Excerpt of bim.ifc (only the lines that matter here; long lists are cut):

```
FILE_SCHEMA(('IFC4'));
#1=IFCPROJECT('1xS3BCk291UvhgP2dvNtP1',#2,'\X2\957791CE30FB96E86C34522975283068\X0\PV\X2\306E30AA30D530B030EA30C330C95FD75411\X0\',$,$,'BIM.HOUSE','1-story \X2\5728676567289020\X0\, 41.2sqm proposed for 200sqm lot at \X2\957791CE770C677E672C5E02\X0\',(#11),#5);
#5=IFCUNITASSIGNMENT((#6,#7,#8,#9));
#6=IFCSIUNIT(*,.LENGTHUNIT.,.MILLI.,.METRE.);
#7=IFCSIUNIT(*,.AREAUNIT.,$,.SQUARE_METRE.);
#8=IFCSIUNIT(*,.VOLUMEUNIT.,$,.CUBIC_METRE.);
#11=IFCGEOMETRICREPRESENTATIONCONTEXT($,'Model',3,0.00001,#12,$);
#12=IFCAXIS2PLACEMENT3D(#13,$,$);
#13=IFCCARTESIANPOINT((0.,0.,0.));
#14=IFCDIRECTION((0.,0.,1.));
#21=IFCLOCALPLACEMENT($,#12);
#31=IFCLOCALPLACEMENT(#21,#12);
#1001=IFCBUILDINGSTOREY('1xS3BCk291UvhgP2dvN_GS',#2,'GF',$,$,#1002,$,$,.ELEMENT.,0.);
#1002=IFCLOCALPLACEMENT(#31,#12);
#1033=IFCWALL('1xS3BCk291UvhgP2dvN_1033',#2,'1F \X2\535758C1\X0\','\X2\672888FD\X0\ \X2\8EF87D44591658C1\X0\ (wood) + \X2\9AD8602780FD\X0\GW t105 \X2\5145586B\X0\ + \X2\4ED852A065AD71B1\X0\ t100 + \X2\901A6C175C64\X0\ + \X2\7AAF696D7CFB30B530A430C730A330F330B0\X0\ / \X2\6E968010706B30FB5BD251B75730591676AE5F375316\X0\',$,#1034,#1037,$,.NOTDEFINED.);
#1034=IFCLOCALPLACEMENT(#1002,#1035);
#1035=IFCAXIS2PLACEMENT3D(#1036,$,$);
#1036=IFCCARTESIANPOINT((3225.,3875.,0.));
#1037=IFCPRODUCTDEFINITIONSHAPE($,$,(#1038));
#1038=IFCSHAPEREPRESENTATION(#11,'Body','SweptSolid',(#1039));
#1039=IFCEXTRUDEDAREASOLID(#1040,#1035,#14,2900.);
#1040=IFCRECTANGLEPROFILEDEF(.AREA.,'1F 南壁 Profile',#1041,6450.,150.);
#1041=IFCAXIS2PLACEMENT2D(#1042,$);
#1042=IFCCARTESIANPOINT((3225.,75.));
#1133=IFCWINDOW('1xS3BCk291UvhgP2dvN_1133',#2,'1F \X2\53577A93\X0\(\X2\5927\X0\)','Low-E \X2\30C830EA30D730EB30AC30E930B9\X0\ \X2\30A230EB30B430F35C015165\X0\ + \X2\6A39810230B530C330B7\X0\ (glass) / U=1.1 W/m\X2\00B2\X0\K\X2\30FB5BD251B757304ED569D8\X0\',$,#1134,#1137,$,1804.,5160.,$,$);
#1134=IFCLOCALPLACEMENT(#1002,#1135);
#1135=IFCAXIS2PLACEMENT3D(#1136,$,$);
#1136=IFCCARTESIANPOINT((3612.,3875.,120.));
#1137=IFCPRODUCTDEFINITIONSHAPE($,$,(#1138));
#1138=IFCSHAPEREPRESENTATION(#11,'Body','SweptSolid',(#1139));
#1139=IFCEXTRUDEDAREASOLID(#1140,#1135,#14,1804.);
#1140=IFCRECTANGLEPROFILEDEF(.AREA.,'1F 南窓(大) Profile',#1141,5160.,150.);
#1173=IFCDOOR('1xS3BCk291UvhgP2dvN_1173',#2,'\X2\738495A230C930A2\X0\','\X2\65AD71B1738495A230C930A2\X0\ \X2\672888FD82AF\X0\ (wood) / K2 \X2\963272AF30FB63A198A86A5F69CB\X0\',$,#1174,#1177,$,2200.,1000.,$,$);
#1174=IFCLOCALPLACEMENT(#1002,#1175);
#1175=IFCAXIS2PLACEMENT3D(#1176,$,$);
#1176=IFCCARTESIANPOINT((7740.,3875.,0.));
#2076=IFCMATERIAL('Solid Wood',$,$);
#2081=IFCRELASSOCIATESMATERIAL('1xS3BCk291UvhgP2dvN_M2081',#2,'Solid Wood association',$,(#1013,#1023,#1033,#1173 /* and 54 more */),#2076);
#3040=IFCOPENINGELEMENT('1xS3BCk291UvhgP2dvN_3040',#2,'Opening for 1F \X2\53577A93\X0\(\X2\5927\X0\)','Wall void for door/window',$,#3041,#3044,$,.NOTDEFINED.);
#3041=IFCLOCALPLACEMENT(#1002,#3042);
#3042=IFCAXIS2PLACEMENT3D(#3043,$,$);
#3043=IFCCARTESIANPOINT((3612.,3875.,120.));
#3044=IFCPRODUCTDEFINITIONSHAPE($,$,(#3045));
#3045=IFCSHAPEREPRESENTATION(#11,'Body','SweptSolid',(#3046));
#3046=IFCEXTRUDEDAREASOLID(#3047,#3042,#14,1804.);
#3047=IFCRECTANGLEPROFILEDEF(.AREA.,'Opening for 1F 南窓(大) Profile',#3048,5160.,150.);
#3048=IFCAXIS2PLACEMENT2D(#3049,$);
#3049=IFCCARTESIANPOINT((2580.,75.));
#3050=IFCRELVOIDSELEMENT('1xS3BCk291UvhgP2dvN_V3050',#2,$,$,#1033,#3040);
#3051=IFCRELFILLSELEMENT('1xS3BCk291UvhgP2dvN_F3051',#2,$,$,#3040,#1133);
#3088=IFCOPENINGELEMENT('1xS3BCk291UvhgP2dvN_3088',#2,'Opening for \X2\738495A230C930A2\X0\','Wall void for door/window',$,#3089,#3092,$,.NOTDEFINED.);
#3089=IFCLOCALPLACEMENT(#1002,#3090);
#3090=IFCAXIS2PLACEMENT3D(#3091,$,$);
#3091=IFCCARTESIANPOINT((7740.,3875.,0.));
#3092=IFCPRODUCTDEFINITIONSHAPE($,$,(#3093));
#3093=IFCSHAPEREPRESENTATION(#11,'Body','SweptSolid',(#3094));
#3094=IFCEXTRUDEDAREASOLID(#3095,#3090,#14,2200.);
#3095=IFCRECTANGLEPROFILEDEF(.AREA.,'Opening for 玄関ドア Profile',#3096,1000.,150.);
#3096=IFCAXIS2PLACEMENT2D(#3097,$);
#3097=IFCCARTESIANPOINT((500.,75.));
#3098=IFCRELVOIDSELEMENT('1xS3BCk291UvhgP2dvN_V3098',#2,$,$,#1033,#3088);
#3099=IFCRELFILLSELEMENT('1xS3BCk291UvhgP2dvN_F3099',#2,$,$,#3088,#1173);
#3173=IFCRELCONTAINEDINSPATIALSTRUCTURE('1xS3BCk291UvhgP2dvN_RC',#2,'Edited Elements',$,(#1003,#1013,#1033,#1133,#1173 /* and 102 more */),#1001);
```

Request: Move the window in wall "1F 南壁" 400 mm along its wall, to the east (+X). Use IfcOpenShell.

```python
import ifcopenshell
import ifcopenshell.api.geometry
import ifcopenshell.util.placement

model = ifcopenshell.open("bim.ifc")

window = model.by_guid("1xS3BCk291UvhgP2dvN_1133")
opening = window.FillsVoids[0].RelatingOpeningElement
wall = opening.VoidsElements[0].RelatingBuildingElement

wall_matrix = ifcopenshell.util.placement.get_local_placement(wall.ObjectPlacement)
shift = wall_matrix[:3, 0] * 400.0
before = ifcopenshell.util.placement.get_local_placement(window.ObjectPlacement)[:3, 3].copy()

# The window is not placed relative to its opening, so move both.
for product in (opening, window):
    matrix = ifcopenshell.util.placement.get_local_placement(product.ObjectPlacement)
    matrix[:3, 3] += shift
    ifcopenshell.api.geometry.edit_object_placement(model, product=product, matrix=matrix, is_si=False)

after = ifcopenshell.util.placement.get_local_placement(window.ObjectPlacement)[:3, 3]
print("window moved by", (after - before).round(3) + 0.0)

model.write("bim_updated.ifc")
```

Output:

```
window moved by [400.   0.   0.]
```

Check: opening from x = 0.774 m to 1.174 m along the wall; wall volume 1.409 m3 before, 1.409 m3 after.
